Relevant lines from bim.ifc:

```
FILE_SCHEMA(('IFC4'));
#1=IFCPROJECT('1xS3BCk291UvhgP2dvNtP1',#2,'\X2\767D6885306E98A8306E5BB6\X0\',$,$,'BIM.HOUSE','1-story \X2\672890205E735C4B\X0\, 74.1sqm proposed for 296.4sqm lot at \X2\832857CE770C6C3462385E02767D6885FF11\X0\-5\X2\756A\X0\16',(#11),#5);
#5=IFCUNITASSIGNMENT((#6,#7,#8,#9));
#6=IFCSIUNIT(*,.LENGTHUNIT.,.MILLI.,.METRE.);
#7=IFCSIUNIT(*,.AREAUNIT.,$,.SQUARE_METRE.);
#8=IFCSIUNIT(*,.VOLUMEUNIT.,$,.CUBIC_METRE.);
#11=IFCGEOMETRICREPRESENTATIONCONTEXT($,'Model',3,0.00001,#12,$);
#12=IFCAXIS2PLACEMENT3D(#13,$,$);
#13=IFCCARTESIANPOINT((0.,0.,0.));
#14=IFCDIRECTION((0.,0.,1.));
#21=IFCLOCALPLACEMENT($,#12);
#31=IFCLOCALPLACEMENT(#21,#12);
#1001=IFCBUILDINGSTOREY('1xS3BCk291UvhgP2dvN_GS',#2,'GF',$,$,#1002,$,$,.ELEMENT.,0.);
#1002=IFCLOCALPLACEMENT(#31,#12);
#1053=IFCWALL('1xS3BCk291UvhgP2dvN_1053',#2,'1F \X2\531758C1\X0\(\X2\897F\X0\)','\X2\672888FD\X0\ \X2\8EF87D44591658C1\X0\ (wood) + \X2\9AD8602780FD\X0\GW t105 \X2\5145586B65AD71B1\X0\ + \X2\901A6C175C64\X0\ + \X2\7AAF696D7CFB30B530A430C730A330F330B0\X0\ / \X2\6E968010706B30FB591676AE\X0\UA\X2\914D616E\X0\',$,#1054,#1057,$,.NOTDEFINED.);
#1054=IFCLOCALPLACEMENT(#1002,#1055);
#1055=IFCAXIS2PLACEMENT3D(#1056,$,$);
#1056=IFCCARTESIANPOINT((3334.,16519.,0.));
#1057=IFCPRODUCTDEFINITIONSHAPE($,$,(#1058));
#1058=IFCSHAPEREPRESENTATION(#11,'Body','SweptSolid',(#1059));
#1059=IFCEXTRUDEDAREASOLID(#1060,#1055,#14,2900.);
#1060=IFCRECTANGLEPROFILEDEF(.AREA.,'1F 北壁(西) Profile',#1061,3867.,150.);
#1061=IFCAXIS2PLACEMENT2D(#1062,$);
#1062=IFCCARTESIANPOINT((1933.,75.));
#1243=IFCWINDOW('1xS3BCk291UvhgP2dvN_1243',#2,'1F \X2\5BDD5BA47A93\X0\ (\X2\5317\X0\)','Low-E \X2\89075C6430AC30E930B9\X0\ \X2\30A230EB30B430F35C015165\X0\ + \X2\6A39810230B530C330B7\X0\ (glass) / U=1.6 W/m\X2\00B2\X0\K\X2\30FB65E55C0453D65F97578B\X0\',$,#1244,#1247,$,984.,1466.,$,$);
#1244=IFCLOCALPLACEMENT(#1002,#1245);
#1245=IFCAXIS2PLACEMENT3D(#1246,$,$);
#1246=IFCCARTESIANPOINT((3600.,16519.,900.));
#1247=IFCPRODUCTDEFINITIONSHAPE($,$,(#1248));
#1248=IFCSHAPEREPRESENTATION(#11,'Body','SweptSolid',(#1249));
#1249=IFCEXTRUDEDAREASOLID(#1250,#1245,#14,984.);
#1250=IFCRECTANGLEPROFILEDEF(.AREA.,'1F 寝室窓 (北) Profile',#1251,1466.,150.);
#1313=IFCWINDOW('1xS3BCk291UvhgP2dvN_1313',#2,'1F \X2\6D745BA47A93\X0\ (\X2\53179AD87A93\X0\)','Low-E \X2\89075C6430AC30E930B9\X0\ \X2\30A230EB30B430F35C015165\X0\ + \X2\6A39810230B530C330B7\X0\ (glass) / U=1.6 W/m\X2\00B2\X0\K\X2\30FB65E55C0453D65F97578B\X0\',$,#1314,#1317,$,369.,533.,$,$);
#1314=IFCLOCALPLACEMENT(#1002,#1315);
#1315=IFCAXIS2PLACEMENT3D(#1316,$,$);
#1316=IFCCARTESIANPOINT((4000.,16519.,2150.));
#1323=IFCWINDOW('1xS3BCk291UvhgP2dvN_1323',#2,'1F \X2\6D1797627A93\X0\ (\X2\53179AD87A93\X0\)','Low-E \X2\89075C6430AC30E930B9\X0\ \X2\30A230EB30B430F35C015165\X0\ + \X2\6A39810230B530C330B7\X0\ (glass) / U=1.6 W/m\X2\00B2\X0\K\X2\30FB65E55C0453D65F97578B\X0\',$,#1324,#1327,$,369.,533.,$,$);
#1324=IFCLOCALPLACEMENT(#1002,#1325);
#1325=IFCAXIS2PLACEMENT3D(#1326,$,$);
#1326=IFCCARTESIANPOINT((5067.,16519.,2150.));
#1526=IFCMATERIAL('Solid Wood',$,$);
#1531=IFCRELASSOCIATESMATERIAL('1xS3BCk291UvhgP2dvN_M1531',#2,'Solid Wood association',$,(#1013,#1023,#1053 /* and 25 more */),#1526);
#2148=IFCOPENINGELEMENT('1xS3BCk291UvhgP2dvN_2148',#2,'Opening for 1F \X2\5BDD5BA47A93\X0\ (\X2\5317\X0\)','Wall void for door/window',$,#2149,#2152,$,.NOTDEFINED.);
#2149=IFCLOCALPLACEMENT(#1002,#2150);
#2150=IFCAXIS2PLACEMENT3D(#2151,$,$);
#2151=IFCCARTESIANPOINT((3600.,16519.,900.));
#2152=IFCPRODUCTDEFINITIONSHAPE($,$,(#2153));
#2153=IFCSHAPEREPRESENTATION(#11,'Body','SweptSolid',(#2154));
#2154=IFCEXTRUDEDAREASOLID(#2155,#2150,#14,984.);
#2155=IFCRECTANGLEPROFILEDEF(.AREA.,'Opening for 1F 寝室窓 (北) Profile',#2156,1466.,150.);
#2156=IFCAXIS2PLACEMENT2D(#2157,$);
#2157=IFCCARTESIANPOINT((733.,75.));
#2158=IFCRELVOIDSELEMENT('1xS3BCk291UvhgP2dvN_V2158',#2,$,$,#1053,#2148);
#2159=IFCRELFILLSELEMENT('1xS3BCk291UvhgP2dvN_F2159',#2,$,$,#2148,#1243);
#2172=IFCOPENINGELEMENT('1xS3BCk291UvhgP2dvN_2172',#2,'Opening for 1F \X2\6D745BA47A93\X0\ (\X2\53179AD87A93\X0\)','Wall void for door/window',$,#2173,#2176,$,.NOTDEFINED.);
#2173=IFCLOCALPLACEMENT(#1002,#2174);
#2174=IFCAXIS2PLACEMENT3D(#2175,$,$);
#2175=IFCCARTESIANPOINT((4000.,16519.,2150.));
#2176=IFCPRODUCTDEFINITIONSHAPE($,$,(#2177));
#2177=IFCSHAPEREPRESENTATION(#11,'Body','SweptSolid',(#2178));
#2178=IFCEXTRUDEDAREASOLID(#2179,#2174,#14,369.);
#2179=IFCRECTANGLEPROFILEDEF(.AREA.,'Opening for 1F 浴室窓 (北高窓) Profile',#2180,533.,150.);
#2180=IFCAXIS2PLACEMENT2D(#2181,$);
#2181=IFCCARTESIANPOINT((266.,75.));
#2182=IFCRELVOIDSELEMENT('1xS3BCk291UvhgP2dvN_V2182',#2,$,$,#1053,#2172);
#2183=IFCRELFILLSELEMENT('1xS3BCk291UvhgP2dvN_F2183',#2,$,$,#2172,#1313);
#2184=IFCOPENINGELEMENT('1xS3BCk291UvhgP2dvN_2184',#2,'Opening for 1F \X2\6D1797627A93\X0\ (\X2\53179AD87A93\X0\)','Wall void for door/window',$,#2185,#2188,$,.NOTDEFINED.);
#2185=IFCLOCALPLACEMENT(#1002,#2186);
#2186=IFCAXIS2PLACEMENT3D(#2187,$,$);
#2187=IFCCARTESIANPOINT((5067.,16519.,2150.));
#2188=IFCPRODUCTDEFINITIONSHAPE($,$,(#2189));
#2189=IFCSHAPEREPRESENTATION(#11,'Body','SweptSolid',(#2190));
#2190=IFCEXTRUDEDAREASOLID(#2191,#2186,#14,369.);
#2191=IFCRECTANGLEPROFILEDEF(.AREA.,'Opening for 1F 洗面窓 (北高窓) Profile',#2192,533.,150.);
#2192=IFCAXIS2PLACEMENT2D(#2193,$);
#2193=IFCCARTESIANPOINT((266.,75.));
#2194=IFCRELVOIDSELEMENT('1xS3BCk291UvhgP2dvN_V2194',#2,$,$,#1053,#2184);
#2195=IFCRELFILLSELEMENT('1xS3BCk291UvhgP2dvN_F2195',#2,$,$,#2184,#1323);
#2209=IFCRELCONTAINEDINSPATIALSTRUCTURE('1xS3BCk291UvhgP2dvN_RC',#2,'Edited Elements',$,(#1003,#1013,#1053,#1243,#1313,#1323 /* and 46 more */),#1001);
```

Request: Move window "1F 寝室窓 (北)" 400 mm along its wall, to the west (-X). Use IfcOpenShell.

```python
import ifcopenshell
import ifcopenshell.api.geometry
import ifcopenshell.util.placement
import ifcopenshell.util.unit

model = ifcopenshell.open("bim.ifc")
unit_scale = ifcopenshell.util.unit.calculate_unit_scale(model)

window = model.by_guid("1xS3BCk291UvhgP2dvN_1243")
opening = window.FillsVoids[0].RelatingOpeningElement
wall = opening.VoidsElements[0].RelatingBuildingElement

wall_matrix = ifcopenshell.util.placement.get_local_placement(wall.ObjectPlacement)
shift = wall_matrix[:3, 0] * -0.4 / unit_scale
before = ifcopenshell.util.placement.get_local_placement(window.ObjectPlacement)[:3, 3].copy()

# The window is not placed relative to its opening, so move both.
for product in (opening, window):
    matrix = ifcopenshell.util.placement.get_local_placement(product.ObjectPlacement)
    matrix[:3, 3] += shift
    ifcopenshell.api.geometry.edit_object_placement(model, product=product, matrix=matrix, is_si=False)

after = ifcopenshell.util.placement.get_local_placement(window.ObjectPlacement)[:3, 3]
print("window moved by", (after - before).round(3) + 0.0)

model.write("bim-out.ifc")
```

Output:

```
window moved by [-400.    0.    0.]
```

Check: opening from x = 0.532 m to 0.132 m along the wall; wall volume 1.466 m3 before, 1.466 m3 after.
